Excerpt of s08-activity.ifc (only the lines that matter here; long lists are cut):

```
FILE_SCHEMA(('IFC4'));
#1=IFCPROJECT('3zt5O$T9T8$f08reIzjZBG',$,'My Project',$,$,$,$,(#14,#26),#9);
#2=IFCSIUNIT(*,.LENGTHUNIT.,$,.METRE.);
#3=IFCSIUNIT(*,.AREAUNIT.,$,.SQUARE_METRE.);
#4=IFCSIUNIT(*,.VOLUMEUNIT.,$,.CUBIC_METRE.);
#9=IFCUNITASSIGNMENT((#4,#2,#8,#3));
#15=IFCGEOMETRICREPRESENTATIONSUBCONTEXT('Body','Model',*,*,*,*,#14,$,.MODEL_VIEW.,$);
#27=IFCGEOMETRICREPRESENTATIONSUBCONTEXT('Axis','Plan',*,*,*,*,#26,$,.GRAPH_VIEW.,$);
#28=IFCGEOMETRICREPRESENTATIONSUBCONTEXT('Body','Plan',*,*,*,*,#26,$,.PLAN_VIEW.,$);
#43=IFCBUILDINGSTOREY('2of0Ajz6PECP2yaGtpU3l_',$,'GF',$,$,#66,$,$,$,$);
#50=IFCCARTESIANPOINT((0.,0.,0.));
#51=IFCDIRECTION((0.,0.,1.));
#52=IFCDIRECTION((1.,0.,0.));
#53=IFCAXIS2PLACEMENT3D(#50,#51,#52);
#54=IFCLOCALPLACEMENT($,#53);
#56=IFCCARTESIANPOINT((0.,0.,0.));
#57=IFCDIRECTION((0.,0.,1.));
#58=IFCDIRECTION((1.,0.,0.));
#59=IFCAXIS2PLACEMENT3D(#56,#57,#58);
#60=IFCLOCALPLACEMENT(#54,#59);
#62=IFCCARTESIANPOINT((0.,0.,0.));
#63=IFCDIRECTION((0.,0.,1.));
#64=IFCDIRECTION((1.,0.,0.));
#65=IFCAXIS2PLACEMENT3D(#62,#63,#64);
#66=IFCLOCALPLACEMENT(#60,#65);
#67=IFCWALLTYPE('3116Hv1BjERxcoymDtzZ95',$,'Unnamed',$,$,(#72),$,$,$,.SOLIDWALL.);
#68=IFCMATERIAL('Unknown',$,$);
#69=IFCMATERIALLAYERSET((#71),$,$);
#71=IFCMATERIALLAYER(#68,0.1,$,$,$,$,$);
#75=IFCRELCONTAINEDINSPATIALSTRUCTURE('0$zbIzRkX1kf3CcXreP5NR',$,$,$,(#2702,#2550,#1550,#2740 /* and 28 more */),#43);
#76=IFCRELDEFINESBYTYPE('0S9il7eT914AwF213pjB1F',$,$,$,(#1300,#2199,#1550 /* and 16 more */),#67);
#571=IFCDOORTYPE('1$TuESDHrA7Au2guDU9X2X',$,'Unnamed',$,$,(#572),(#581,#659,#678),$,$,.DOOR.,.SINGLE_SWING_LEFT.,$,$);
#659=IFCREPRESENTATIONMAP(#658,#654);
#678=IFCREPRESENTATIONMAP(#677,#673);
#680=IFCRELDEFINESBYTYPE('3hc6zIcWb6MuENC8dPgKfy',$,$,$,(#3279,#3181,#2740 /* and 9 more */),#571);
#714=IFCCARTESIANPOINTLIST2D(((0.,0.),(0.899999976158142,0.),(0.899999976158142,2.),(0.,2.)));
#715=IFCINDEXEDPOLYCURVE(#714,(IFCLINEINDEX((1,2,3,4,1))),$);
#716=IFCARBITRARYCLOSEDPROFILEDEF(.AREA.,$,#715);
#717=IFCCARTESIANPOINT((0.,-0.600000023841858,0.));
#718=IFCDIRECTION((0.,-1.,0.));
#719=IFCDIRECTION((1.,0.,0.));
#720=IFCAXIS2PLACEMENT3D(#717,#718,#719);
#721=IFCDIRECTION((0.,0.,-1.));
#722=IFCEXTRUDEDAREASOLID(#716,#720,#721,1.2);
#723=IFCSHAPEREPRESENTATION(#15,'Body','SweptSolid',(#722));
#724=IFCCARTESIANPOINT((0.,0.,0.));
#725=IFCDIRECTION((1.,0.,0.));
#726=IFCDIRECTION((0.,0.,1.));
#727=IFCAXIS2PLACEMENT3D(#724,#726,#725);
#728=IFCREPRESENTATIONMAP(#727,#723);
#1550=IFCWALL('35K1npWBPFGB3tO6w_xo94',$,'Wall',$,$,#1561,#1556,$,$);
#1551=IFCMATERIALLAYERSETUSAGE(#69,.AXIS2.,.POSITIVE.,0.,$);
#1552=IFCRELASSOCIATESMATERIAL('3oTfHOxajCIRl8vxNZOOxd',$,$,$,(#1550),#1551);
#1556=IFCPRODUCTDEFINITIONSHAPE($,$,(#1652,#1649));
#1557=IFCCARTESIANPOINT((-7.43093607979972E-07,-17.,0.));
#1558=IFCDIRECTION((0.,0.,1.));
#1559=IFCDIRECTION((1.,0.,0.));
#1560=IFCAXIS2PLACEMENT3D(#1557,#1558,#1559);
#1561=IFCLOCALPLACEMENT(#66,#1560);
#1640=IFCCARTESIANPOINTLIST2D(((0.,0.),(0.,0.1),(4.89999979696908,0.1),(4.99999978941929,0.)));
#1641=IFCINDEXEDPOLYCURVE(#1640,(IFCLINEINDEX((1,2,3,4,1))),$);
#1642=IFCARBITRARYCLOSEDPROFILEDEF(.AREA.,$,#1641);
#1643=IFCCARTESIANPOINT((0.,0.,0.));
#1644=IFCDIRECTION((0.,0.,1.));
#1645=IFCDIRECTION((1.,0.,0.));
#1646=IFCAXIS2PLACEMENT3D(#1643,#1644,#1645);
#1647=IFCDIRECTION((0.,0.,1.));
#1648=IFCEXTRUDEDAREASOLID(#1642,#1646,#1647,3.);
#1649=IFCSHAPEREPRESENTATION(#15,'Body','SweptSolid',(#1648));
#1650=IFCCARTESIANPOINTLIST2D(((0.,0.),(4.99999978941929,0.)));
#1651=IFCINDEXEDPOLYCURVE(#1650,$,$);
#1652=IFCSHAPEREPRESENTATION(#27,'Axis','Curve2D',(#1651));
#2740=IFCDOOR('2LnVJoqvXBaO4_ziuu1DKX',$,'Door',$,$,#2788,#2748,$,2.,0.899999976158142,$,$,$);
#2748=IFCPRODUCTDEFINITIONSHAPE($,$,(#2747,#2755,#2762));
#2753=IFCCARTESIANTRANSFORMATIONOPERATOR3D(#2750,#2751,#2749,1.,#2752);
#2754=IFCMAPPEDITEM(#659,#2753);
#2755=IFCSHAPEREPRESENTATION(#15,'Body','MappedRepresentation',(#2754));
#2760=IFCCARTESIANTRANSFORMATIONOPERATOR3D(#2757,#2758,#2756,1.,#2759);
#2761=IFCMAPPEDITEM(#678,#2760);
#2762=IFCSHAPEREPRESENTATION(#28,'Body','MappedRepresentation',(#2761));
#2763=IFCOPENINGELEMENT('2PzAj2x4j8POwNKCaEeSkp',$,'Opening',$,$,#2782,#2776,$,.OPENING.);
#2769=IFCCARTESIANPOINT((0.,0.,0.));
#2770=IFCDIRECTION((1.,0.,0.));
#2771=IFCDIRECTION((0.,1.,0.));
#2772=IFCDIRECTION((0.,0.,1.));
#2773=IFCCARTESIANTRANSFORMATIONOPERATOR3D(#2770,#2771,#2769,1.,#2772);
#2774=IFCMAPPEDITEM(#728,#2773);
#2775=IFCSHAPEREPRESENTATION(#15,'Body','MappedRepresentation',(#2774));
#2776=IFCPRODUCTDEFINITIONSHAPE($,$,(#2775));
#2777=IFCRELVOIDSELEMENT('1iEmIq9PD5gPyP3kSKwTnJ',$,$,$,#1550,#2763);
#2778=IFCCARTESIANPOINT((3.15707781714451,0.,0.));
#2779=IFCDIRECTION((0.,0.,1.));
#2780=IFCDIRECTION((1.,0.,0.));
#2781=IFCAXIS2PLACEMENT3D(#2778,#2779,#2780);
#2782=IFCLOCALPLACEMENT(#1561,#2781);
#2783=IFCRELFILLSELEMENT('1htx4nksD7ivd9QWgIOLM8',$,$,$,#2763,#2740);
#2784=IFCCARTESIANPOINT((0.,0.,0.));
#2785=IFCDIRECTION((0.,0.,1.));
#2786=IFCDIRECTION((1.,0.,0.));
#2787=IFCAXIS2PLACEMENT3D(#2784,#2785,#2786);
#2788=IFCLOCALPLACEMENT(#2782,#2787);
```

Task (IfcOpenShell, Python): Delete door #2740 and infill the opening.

```python
import ifcopenshell
import ifcopenshell.api.feature
import ifcopenshell.api.root
import ifcopenshell.geom
import ifcopenshell.util.shape

model = ifcopenshell.open("s08-activity.ifc")
settings = ifcopenshell.geom.settings()


def volume(element):
    """Net volume in cubic metres, openings subtracted."""
    shape = ifcopenshell.geom.create_shape(settings, element)
    return ifcopenshell.util.shape.get_volume(shape.geometry)


door = model.by_guid("2LnVJoqvXBaO4_ziuu1DKX")
opening = door.FillsVoids[0].RelatingOpeningElement
wall = opening.VoidsElements[0].RelatingBuildingElement
before = volume(wall)

ifcopenshell.api.root.remove_product(model, product=door)
ifcopenshell.api.feature.remove_feature(model, feature=opening)

after = volume(wall)

print(f"wall volume {before:.3f} -> {after:.3f} m3")

model.write("s08-activity_edited.ifc")
```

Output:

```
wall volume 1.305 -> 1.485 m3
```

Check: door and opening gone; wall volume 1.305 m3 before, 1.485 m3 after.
